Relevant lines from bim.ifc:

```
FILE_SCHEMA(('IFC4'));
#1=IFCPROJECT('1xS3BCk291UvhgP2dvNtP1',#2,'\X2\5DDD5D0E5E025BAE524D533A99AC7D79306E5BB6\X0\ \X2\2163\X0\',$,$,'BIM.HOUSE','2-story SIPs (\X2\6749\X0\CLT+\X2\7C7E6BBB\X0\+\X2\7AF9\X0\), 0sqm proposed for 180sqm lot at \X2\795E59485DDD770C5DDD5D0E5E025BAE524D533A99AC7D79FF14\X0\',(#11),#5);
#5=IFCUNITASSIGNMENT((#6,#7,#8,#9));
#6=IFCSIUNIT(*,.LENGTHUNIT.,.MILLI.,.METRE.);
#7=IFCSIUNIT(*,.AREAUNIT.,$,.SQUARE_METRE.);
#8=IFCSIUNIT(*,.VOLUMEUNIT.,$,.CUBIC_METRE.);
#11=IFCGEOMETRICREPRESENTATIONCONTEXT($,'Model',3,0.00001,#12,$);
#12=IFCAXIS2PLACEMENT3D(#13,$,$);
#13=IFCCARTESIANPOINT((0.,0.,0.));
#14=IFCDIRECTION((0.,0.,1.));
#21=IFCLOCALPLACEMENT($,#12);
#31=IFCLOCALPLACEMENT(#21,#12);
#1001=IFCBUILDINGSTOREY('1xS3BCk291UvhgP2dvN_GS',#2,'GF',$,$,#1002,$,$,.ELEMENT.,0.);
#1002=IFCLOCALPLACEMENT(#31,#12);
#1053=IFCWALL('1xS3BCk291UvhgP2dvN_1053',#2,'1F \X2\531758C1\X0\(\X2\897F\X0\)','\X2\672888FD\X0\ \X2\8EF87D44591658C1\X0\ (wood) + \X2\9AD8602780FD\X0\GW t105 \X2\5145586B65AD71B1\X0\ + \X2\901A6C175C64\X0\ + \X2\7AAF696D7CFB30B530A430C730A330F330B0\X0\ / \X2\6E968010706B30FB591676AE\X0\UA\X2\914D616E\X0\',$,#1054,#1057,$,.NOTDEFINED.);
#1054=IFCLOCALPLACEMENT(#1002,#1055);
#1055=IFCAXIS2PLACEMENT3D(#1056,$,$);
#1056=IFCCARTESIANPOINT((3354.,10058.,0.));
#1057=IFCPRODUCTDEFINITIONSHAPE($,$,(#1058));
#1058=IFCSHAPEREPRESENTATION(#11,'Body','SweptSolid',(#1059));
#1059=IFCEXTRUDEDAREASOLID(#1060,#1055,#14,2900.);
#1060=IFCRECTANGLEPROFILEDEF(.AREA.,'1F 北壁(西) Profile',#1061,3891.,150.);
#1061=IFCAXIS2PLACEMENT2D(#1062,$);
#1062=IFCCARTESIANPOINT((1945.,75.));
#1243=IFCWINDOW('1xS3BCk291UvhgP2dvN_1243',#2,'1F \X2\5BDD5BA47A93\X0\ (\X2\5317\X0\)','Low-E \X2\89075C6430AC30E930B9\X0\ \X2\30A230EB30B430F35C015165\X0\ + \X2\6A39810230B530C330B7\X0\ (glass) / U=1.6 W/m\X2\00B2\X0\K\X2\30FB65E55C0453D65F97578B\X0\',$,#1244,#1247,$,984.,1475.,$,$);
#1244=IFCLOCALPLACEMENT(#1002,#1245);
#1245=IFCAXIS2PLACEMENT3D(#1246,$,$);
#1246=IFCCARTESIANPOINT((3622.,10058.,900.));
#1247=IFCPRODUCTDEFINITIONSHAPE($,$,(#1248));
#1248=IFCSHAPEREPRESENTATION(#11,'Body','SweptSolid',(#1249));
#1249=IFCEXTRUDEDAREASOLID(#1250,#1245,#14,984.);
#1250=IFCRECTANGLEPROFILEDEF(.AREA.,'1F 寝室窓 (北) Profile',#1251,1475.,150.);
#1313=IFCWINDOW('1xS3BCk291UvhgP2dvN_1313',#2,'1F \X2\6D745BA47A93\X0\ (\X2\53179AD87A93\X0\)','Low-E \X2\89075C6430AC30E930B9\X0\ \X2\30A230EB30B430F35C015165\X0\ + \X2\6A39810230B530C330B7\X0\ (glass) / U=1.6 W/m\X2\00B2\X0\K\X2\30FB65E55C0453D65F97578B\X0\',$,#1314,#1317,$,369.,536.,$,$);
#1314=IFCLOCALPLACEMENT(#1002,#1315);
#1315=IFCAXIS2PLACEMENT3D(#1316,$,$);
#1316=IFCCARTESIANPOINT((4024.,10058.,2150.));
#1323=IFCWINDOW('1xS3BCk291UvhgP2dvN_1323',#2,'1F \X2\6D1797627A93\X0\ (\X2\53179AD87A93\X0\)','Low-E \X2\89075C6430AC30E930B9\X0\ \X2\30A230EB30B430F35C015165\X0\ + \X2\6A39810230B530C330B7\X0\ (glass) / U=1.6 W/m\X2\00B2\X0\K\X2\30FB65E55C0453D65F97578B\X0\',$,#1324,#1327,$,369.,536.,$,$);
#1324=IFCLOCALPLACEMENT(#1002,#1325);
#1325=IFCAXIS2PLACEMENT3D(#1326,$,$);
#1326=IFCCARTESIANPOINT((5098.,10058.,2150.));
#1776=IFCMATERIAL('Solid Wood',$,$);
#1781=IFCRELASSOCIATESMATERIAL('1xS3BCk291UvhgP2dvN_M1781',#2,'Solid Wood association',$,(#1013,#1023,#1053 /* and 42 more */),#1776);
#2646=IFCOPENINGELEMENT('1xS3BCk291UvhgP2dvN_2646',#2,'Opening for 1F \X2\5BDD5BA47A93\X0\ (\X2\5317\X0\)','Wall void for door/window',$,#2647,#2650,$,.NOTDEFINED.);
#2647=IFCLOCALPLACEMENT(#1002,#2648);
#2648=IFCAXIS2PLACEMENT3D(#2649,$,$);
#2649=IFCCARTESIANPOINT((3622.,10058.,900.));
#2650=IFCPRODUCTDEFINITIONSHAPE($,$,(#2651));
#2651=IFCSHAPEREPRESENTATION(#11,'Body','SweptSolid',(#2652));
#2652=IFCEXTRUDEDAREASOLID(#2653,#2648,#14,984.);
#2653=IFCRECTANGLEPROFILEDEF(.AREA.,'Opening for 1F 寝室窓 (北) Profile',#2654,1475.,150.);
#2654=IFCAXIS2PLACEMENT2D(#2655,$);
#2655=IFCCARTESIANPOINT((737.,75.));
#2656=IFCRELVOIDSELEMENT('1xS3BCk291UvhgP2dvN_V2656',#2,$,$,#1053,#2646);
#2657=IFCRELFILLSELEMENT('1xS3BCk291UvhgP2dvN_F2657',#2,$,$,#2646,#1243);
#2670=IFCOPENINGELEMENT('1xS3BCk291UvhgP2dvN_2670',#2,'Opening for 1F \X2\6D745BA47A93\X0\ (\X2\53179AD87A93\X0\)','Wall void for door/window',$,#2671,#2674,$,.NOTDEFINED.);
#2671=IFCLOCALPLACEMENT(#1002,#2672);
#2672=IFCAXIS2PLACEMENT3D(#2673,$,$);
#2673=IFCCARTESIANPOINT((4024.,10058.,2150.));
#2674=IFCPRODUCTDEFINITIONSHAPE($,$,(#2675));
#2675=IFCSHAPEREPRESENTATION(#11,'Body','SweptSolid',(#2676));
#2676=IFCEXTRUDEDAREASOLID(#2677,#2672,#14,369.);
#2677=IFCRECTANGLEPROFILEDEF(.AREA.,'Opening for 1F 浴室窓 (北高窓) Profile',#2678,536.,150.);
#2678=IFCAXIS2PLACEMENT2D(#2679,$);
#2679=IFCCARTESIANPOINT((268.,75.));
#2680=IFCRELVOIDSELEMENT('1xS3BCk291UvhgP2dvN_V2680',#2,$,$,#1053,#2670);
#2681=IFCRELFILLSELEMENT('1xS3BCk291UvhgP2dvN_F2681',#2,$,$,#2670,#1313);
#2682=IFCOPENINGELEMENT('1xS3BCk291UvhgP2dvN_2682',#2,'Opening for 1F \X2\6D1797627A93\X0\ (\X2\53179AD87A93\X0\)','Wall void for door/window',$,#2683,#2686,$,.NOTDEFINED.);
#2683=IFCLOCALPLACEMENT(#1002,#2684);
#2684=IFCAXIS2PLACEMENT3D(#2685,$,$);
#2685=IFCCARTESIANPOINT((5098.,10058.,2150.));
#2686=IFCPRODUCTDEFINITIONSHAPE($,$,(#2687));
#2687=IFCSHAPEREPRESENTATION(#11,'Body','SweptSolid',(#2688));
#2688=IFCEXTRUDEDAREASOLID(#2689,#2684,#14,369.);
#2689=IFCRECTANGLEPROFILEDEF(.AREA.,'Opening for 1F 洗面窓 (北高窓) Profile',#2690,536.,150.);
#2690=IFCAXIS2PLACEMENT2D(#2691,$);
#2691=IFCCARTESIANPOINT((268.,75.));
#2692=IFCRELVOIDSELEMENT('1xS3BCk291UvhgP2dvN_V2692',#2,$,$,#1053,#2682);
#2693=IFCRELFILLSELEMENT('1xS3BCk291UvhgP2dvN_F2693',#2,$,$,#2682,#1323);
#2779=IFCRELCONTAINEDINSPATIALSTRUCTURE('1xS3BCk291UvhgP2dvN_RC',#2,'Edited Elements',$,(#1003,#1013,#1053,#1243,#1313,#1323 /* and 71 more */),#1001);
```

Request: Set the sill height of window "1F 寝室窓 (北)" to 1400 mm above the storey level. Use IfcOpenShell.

```python
import numpy as np
import ifcopenshell
import ifcopenshell.api.geometry
import ifcopenshell.geom
import ifcopenshell.util.element
import ifcopenshell.util.placement
import ifcopenshell.util.shape
import ifcopenshell.util.unit

model = ifcopenshell.open("bim.ifc")
unit_scale = ifcopenshell.util.unit.calculate_unit_scale(model)

window = model.by_guid("1xS3BCk291UvhgP2dvN_1243")
opening = window.FillsVoids[0].RelatingOpeningElement
storey = ifcopenshell.util.element.get_container(window, ifc_class="IfcBuildingStorey")
level = ifcopenshell.util.placement.get_local_placement(storey.ObjectPlacement)[2, 3]

# The opening's origin need not be at the sill, so measure its lowest point.
shape = ifcopenshell.geom.create_shape(ifcopenshell.geom.settings(), opening)
bottom = ifcopenshell.util.shape.get_shape_bottom_elevation(shape, shape.geometry) / unit_scale
dz = level + 1400.0 - bottom

shift = np.array([0.0, 0.0, dz])
# The window is not placed relative to its opening, so move both.
for product in (opening, window):
    matrix = ifcopenshell.util.placement.get_local_placement(product.ObjectPlacement)
    matrix[:3, 3] += shift
    ifcopenshell.api.geometry.edit_object_placement(model, product=product, matrix=matrix, is_si=False)

print(f"moved by {dz * unit_scale:+.3f} m")

model.write("bim_v2.ifc")
```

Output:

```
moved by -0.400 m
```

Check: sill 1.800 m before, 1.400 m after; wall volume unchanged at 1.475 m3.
